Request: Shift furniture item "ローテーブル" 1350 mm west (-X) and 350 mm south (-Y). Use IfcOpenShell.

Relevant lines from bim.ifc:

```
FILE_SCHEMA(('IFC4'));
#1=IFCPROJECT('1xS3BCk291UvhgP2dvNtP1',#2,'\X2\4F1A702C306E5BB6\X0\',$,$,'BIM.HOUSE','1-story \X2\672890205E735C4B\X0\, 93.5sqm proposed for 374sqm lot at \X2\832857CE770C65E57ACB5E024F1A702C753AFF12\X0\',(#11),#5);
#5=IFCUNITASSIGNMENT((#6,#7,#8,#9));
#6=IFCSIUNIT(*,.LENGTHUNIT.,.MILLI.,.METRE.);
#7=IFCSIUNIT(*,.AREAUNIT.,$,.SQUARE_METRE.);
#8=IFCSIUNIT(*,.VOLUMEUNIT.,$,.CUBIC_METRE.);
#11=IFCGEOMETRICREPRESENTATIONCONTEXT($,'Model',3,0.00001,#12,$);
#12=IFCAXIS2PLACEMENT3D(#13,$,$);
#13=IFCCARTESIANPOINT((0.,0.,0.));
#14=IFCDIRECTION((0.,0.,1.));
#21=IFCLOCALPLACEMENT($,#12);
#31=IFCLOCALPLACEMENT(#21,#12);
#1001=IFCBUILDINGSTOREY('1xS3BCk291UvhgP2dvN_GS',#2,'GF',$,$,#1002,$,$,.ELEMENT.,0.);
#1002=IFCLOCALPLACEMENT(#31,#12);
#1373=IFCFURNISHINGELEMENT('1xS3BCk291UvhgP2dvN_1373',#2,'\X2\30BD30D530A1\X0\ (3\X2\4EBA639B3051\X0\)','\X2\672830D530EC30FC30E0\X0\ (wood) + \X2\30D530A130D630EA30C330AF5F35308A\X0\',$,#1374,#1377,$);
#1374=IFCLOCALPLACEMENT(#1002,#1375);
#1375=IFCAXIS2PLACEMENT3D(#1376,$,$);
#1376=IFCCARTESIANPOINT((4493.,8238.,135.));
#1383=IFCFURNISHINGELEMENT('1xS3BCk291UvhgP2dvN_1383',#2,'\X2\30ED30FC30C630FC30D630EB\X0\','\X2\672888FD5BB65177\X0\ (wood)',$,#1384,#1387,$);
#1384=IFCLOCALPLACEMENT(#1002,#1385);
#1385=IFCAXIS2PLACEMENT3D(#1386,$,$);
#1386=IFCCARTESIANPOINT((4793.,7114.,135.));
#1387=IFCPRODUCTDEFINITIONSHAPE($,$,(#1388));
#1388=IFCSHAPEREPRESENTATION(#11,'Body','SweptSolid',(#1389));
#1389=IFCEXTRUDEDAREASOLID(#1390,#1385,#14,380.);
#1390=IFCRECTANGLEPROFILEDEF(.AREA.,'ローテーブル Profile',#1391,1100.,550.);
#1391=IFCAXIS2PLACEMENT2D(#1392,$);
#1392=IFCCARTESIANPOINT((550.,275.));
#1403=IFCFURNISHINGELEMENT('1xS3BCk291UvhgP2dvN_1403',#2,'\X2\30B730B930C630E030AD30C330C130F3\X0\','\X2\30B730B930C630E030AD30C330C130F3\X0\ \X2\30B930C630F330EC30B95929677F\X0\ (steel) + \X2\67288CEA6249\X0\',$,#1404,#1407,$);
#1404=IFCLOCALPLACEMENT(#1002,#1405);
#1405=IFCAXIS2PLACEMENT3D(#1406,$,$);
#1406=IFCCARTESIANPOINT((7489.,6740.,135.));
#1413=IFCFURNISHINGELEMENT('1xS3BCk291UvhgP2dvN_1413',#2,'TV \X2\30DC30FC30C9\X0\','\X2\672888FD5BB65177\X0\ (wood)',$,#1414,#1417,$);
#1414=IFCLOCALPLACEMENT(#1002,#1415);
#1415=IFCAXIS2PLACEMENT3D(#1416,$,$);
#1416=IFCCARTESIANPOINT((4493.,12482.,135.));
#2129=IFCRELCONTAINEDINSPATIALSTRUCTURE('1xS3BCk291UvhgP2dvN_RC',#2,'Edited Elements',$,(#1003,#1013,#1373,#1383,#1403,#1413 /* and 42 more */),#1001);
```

```python
import ifcopenshell
import ifcopenshell.api.geometry
import ifcopenshell.util.placement

model = ifcopenshell.open("bim.ifc")

item = model.by_id(1383)
matrix = ifcopenshell.util.placement.get_local_placement(item.ObjectPlacement)
matrix[0, 3] -= 1350.0
matrix[1, 3] -= 350.0
ifcopenshell.api.geometry.edit_object_placement(model, product=item, matrix=matrix, is_si=False)

print(ifcopenshell.util.placement.get_local_placement(item.ObjectPlacement).round(3) + 0.0)

model.write("bim-out.ifc")
```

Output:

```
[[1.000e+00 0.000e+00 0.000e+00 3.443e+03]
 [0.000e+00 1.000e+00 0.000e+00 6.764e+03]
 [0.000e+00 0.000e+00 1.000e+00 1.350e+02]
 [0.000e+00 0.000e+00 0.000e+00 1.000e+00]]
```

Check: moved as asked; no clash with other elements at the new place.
